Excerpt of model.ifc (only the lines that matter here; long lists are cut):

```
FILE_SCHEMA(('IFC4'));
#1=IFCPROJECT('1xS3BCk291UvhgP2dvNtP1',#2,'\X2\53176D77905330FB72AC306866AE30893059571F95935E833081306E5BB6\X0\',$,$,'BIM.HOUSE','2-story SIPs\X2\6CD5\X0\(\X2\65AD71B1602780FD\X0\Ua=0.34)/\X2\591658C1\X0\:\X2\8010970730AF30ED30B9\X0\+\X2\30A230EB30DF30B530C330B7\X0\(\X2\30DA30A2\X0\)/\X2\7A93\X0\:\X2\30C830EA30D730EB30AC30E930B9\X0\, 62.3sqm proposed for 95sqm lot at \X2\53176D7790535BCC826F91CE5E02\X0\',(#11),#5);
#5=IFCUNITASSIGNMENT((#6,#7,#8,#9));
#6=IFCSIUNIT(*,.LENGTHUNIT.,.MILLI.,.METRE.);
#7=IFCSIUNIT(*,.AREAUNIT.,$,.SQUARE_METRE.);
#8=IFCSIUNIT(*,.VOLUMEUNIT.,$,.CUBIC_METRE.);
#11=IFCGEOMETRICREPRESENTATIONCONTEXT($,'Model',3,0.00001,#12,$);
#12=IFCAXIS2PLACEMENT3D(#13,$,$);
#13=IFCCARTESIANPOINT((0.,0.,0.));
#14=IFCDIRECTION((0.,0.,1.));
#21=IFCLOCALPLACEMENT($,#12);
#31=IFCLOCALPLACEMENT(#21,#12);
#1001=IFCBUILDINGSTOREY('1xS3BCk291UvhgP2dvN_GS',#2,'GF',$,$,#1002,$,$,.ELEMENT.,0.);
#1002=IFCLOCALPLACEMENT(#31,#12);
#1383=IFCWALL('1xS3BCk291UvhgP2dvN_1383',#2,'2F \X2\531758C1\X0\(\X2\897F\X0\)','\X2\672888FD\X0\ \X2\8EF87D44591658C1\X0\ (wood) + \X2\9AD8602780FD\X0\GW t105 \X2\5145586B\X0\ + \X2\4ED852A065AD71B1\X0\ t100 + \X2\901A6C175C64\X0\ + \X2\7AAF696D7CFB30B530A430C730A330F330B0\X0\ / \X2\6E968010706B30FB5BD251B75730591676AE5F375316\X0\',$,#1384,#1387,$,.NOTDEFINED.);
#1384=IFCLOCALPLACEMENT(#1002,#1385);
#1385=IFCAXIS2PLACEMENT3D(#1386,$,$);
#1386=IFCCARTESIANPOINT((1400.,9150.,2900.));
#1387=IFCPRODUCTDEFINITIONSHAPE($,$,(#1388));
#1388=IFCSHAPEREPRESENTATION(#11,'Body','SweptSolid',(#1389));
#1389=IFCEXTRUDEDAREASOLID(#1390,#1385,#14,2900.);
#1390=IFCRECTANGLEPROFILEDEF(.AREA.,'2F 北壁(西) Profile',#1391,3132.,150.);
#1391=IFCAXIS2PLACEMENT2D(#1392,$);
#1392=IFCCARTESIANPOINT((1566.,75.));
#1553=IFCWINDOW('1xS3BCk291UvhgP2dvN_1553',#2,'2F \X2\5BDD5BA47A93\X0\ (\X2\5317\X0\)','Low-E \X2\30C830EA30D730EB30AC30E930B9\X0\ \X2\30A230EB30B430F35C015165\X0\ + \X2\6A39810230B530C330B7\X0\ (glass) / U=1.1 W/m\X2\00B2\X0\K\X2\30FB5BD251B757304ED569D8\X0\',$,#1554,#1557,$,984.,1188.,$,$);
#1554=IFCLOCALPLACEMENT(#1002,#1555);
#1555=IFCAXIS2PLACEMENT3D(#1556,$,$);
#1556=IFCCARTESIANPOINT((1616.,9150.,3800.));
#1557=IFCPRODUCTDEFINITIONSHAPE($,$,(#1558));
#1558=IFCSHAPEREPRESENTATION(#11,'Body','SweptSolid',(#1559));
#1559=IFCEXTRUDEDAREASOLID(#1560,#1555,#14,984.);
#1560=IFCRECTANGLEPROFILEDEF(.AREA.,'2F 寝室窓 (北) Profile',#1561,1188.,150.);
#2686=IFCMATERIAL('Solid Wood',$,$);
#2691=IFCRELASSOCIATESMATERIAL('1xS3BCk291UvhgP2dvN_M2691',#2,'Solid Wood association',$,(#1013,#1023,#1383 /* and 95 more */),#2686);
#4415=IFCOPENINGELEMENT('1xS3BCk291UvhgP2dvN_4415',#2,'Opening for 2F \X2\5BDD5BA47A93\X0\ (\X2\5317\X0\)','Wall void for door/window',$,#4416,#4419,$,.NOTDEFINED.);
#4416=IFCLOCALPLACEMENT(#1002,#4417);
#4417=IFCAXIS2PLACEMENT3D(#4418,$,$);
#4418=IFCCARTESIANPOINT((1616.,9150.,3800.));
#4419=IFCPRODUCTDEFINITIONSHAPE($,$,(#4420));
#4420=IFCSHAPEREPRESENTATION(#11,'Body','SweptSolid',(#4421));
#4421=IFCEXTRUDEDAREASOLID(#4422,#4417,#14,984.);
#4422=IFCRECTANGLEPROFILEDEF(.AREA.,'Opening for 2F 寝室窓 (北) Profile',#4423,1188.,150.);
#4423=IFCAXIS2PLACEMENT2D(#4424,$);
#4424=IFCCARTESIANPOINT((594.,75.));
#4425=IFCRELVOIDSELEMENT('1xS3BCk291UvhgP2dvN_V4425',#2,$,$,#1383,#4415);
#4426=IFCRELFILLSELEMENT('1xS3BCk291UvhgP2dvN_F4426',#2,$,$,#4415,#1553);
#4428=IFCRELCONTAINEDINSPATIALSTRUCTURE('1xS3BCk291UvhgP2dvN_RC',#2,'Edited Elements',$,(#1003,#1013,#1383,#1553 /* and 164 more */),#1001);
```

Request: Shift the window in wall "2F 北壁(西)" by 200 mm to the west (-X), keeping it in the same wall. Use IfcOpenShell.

```python
import ifcopenshell
import ifcopenshell.api.geometry
import ifcopenshell.util.placement

model = ifcopenshell.open("model.ifc")

window = model.by_id(1553)
opening = window.FillsVoids[0].RelatingOpeningElement
wall = opening.VoidsElements[0].RelatingBuildingElement

wall_matrix = ifcopenshell.util.placement.get_local_placement(wall.ObjectPlacement)
shift = wall_matrix[:3, 0] * -200.0
before = ifcopenshell.util.placement.get_local_placement(window.ObjectPlacement)[:3, 3].copy()

# The window is not placed relative to its opening, so move both.
for product in (opening, window):
    matrix = ifcopenshell.util.placement.get_local_placement(product.ObjectPlacement)
    matrix[:3, 3] += shift
    ifcopenshell.api.geometry.edit_object_placement(model, product=product, matrix=matrix, is_si=False)

after = ifcopenshell.util.placement.get_local_placement(window.ObjectPlacement)[:3, 3]
print("window moved by", (after - before).round(3) + 0.0)

model.write("model_rev.ifc")
```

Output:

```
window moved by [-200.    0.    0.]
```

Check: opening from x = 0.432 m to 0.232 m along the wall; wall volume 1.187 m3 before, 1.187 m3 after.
